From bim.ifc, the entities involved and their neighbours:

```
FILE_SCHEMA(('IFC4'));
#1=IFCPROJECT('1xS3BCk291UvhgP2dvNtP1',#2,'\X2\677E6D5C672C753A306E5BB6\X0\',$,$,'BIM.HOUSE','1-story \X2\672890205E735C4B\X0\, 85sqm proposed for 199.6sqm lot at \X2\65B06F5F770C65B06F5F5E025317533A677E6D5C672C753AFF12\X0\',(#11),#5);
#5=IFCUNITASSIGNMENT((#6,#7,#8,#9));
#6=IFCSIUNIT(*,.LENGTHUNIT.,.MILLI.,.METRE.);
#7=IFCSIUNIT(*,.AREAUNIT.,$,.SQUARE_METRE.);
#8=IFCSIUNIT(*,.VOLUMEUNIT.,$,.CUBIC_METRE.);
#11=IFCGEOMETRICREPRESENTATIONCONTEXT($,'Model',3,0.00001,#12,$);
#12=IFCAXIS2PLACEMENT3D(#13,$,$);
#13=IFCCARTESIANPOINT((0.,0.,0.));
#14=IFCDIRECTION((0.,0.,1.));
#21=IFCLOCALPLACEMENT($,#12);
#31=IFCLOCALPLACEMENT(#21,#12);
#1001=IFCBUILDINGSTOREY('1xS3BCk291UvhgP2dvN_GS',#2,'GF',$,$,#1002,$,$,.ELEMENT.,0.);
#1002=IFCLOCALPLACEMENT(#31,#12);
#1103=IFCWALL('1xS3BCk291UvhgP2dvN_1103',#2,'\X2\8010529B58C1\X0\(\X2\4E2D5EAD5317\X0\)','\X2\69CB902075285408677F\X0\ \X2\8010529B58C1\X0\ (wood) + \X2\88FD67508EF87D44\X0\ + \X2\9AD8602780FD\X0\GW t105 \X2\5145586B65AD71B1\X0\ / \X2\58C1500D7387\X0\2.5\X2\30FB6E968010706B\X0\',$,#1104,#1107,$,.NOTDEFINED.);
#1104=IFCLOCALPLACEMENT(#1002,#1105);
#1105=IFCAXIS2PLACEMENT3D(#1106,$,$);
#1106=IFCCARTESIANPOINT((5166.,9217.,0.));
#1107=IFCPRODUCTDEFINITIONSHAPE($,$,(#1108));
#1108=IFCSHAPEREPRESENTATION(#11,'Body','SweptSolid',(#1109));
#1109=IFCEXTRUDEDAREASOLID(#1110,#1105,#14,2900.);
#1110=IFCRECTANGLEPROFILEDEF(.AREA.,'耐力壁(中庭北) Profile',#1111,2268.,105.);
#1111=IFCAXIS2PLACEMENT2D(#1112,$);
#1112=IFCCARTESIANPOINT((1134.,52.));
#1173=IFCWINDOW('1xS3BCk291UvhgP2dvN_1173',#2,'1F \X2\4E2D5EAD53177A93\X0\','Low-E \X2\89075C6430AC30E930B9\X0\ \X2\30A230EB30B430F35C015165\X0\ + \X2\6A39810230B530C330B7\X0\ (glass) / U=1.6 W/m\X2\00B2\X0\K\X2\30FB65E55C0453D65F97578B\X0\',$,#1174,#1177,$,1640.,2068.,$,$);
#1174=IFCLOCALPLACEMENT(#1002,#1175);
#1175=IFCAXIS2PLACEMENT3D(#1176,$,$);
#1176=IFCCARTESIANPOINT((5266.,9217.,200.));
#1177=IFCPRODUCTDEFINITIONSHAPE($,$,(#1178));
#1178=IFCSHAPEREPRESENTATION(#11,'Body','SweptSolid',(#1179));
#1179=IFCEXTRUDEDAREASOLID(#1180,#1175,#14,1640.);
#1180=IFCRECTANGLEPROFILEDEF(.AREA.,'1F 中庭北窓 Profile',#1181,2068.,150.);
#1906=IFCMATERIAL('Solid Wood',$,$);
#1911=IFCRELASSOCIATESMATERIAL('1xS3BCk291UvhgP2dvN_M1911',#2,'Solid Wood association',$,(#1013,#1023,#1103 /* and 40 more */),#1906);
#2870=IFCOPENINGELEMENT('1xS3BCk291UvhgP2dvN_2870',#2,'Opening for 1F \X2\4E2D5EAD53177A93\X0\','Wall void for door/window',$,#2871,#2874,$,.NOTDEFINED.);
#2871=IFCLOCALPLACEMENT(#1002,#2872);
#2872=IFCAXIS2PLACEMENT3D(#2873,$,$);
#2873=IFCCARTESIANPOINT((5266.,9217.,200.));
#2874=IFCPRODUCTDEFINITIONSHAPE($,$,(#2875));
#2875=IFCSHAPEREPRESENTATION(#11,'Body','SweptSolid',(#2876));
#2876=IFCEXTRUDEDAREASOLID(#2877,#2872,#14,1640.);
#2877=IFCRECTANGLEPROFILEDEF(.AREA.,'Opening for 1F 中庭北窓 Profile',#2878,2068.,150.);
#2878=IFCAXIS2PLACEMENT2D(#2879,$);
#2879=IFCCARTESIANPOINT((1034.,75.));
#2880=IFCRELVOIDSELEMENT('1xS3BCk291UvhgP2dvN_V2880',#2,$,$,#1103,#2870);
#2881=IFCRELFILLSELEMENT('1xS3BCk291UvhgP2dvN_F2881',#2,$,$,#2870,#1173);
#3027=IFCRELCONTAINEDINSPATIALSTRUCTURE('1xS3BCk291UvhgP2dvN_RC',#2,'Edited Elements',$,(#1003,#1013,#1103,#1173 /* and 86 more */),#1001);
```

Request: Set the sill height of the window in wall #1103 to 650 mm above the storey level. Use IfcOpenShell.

```python
import numpy as np
import ifcopenshell
import ifcopenshell.api.geometry
import ifcopenshell.geom
import ifcopenshell.util.element
import ifcopenshell.util.placement
import ifcopenshell.util.shape
import ifcopenshell.util.unit

model = ifcopenshell.open("bim.ifc")
unit_scale = ifcopenshell.util.unit.calculate_unit_scale(model)

window = model.by_guid("1xS3BCk291UvhgP2dvN_1173")
opening = window.FillsVoids[0].RelatingOpeningElement
storey = ifcopenshell.util.element.get_container(window, ifc_class="IfcBuildingStorey")
level = ifcopenshell.util.placement.get_local_placement(storey.ObjectPlacement)[2, 3]

# The opening's origin need not be at the sill, so measure its lowest point.
shape = ifcopenshell.geom.create_shape(ifcopenshell.geom.settings(), opening)
bottom = ifcopenshell.util.shape.get_shape_bottom_elevation(shape, shape.geometry) / unit_scale
dz = level + 0.65 / unit_scale - bottom

shift = np.array([0.0, 0.0, dz])
# The window is not placed relative to its opening, so move both.
for product in (opening, window):
    matrix = ifcopenshell.util.placement.get_local_placement(product.ObjectPlacement)
    matrix[:3, 3] += shift
    ifcopenshell.api.geometry.edit_object_placement(model, product=product, matrix=matrix, is_si=False)

print(f"moved by {dz * unit_scale:+.3f} m")

model.write("bim_v2.ifc")
```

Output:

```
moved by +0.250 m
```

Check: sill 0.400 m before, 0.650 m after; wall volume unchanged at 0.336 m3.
